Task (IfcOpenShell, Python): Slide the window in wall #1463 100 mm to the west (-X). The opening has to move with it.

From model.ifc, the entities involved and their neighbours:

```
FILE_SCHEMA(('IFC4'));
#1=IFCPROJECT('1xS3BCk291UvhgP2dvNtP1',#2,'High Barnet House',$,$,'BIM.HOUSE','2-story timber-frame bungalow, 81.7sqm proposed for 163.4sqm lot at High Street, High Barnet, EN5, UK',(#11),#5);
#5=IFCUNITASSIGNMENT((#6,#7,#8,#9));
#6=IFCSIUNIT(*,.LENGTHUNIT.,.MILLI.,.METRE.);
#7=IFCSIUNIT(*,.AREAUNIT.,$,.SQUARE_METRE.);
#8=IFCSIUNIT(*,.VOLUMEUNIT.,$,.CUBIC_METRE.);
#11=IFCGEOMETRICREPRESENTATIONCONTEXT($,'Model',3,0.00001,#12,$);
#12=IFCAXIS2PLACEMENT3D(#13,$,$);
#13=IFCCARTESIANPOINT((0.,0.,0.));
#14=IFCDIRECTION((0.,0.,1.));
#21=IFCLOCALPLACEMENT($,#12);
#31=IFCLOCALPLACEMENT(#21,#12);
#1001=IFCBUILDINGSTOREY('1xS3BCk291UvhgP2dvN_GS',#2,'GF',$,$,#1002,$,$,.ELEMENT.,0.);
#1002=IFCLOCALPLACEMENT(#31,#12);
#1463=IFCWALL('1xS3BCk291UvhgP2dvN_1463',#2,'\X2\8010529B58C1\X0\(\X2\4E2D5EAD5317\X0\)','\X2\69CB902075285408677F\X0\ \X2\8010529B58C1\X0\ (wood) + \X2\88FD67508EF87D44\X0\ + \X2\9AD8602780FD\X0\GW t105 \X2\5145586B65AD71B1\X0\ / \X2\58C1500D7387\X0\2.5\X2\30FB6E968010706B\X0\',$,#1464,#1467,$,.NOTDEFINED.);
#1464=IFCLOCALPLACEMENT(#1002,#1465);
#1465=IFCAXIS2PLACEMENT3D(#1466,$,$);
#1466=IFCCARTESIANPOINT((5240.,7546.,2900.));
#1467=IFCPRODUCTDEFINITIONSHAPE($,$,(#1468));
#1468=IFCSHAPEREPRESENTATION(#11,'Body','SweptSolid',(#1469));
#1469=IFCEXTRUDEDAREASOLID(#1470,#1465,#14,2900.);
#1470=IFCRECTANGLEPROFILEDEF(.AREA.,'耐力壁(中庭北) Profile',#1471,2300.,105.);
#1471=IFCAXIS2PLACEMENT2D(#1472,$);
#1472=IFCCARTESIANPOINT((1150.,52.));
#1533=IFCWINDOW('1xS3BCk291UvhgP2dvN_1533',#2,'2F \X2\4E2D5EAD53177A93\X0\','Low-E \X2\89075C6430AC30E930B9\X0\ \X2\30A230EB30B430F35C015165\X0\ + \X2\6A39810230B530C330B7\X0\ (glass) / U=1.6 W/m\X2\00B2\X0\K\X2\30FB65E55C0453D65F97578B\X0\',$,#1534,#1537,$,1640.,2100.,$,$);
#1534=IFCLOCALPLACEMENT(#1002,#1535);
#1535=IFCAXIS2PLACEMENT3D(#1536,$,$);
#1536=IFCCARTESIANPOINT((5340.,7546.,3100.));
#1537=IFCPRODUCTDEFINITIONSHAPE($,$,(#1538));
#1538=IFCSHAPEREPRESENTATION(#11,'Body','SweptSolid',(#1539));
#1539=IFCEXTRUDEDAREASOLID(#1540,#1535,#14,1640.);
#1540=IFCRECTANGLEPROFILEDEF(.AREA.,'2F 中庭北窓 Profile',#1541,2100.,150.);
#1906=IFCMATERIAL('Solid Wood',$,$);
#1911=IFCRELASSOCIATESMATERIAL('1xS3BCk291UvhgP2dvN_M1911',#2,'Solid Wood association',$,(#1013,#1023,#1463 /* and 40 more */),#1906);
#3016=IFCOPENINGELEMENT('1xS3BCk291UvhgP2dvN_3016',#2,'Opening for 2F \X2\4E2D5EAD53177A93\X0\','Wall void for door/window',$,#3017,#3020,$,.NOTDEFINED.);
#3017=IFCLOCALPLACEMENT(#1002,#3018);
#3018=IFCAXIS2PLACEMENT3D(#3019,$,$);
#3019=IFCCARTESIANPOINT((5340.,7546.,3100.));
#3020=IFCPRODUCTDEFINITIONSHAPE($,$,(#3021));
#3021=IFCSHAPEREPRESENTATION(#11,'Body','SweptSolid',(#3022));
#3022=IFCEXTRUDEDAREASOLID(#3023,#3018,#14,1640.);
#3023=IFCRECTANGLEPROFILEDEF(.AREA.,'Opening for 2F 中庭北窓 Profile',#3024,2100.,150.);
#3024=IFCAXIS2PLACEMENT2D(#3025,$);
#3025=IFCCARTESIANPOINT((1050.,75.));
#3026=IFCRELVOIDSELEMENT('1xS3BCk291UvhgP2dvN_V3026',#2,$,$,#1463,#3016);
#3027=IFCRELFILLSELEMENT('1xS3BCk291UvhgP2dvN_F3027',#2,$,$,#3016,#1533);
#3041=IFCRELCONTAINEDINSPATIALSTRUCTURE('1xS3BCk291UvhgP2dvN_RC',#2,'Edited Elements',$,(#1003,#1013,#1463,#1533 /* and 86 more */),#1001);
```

```python
import ifcopenshell
import ifcopenshell.api.geometry
import ifcopenshell.util.placement
import ifcopenshell.util.unit

model = ifcopenshell.open("model.ifc")
unit_scale = ifcopenshell.util.unit.calculate_unit_scale(model)

window = model.by_guid("1xS3BCk291UvhgP2dvN_1533")
opening = window.FillsVoids[0].RelatingOpeningElement
wall = opening.VoidsElements[0].RelatingBuildingElement

wall_matrix = ifcopenshell.util.placement.get_local_placement(wall.ObjectPlacement)
shift = wall_matrix[:3, 0] * -0.1 / unit_scale
before = ifcopenshell.util.placement.get_local_placement(window.ObjectPlacement)[:3, 3].copy()

# The window is not placed relative to its opening, so move both.
for product in (opening, window):
    matrix = ifcopenshell.util.placement.get_local_placement(product.ObjectPlacement)
    matrix[:3, 3] += shift
    ifcopenshell.api.geometry.edit_object_placement(model, product=product, matrix=matrix, is_si=False)

after = ifcopenshell.util.placement.get_local_placement(window.ObjectPlacement)[:3, 3]
print("window moved by", (after - before).round(3) + 0.0)

model.write("model_rev.ifc")
```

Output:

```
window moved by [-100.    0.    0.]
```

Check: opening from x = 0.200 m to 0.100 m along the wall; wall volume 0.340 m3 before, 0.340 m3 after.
